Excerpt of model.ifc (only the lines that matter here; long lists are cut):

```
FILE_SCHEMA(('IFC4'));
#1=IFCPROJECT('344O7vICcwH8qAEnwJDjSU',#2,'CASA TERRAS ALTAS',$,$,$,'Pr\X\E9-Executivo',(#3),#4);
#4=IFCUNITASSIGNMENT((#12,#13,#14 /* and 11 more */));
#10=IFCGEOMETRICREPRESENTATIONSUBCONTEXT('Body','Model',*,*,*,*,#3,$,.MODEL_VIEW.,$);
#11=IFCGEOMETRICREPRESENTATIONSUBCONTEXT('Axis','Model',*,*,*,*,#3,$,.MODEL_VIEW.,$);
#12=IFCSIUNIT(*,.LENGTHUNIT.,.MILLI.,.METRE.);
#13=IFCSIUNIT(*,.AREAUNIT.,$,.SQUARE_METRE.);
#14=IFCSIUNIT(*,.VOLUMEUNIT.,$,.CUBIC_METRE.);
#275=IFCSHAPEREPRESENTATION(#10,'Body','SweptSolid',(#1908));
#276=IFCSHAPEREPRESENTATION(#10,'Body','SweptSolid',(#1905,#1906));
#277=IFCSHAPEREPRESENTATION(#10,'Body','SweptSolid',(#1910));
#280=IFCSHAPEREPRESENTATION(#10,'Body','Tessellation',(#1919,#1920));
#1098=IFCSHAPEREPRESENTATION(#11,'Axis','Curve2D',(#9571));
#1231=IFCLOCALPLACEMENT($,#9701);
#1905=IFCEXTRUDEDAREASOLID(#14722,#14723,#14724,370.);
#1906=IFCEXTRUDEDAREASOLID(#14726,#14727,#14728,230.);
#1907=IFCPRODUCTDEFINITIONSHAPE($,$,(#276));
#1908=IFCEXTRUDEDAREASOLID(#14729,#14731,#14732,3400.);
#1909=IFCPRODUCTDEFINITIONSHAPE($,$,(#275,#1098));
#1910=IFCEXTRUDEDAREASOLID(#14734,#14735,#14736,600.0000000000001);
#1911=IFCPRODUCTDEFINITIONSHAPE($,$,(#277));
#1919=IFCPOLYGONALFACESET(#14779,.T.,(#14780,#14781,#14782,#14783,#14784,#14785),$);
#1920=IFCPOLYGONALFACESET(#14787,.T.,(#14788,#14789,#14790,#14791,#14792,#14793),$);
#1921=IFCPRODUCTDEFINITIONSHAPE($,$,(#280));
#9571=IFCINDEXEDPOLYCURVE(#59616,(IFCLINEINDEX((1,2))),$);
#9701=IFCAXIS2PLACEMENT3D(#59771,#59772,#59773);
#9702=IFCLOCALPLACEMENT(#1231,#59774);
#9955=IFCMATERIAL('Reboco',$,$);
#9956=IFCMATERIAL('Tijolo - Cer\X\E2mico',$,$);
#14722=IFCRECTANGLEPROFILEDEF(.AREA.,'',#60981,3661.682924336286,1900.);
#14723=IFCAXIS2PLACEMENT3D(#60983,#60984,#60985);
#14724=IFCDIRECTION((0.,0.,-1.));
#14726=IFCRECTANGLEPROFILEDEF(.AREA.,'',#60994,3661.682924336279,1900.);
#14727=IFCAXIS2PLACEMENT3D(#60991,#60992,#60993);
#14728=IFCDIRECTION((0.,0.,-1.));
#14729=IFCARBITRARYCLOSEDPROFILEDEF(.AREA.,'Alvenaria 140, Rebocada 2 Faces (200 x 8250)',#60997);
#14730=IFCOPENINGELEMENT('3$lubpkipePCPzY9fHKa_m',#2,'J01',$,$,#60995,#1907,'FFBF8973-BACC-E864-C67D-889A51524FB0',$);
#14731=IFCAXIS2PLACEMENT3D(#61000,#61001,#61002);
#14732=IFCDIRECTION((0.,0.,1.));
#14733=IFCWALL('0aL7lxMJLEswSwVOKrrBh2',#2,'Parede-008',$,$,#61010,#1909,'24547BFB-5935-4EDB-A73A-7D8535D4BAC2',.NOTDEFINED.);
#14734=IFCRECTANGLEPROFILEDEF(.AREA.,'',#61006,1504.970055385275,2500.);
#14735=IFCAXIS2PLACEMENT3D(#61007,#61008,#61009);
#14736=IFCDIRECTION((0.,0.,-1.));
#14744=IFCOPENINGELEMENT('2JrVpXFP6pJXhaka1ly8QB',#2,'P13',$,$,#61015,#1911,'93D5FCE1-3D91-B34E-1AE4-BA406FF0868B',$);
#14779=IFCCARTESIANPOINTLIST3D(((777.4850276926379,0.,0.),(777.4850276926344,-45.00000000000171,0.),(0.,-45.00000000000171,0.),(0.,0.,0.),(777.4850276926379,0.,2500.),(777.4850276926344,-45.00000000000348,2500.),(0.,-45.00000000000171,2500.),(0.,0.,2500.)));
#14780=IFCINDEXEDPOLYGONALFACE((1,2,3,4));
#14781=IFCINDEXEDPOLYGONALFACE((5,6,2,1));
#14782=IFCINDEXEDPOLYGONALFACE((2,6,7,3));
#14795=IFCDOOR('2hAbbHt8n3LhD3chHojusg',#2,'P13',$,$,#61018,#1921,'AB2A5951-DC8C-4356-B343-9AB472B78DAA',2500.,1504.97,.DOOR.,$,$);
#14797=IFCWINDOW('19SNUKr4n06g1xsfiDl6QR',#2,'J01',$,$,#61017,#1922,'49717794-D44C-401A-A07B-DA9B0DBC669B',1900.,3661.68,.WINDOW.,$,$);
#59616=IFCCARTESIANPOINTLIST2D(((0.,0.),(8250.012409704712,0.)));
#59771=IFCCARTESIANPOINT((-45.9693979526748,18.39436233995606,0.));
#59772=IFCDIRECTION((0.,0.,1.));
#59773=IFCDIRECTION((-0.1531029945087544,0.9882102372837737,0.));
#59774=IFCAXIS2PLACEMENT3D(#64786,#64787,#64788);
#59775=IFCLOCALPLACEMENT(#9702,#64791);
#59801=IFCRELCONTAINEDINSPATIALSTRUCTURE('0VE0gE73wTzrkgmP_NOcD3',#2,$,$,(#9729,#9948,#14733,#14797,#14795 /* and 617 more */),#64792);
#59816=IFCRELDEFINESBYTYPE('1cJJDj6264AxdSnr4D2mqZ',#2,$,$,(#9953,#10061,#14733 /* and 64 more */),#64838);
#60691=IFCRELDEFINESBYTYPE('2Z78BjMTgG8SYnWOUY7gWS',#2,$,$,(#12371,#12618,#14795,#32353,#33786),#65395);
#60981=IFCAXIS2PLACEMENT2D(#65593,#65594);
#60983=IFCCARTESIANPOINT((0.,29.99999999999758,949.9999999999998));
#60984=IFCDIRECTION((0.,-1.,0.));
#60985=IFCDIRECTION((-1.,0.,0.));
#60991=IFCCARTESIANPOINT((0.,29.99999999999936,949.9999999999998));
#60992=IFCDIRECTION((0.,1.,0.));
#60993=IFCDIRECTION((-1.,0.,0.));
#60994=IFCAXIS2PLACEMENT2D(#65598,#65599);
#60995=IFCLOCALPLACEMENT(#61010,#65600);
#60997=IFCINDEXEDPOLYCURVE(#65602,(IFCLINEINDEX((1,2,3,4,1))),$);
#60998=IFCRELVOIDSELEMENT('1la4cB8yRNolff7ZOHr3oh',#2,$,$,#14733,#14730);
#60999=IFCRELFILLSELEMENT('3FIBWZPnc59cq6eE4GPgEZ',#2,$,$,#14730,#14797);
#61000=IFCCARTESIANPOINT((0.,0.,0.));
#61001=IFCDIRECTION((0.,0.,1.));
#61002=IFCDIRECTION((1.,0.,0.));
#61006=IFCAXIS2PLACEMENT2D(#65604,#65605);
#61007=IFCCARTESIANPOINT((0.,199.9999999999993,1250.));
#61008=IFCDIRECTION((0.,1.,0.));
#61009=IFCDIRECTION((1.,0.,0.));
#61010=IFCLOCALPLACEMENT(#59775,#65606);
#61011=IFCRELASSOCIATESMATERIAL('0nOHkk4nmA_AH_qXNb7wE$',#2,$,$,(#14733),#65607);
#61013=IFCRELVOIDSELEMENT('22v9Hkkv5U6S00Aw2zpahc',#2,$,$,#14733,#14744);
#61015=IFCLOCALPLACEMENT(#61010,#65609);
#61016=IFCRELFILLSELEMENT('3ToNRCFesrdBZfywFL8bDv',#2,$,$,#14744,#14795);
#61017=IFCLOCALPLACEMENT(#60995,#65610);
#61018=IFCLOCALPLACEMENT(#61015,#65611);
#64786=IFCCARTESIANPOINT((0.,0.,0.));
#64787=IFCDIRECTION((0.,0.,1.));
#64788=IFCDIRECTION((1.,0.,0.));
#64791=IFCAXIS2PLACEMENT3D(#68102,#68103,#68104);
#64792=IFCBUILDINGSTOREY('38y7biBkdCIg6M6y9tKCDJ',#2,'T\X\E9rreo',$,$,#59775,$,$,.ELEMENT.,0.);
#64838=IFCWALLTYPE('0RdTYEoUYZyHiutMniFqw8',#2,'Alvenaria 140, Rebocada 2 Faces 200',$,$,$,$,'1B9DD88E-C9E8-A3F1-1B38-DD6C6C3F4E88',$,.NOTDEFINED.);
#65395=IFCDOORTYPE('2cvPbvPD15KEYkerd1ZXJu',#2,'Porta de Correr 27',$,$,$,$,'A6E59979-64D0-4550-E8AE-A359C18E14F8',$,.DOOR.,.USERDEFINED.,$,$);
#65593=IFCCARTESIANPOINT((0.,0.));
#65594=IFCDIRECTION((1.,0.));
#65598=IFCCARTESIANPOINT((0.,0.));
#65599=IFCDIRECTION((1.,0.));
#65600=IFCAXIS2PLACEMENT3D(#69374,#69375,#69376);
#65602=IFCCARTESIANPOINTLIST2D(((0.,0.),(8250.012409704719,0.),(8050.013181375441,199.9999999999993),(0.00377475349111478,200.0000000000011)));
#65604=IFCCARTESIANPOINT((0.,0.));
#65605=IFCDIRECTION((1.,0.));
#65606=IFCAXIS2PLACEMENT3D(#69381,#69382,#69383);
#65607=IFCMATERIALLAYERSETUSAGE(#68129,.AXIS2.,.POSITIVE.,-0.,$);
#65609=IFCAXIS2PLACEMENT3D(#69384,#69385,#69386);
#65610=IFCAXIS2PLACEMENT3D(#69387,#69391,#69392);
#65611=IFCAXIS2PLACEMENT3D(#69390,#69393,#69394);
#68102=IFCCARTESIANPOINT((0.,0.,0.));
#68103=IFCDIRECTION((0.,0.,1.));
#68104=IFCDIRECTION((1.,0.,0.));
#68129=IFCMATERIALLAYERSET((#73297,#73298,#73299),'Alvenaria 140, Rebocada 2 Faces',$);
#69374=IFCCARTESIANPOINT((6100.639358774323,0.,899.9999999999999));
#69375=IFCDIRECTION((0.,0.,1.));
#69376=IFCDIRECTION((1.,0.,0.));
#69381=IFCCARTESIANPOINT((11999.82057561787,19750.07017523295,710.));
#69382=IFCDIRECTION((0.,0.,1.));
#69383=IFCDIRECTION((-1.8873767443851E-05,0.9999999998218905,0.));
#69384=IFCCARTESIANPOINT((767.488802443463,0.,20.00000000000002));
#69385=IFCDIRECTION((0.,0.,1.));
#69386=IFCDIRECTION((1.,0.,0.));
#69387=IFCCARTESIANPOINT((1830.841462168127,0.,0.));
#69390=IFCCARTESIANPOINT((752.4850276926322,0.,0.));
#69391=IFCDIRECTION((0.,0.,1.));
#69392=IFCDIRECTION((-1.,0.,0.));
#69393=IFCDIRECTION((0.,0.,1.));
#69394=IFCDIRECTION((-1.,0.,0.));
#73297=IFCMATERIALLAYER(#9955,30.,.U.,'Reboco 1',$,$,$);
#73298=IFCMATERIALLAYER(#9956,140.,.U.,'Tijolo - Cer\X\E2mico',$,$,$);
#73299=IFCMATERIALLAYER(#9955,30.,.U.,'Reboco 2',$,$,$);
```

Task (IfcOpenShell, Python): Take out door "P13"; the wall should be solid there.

```python
import ifcopenshell
import ifcopenshell.api.feature
import ifcopenshell.api.root
import ifcopenshell.geom
import ifcopenshell.util.shape

model = ifcopenshell.open("model.ifc")
settings = ifcopenshell.geom.settings()


def volume(element):
    """Net volume in cubic metres, openings subtracted."""
    shape = ifcopenshell.geom.create_shape(settings, element)
    return ifcopenshell.util.shape.get_volume(shape.geometry)


door = model.by_guid("2hAbbHt8n3LhD3chHojusg")
opening = door.FillsVoids[0].RelatingOpeningElement
wall = opening.VoidsElements[0].RelatingBuildingElement
before = volume(wall)

ifcopenshell.api.root.remove_product(model, product=door)
ifcopenshell.api.feature.remove_feature(model, feature=opening)

after = volume(wall)

print(f"wall volume {before:.3f} -> {after:.3f} m3")

model.write("model_edited.ifc")
```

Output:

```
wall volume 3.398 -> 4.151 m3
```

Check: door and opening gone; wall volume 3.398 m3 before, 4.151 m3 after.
